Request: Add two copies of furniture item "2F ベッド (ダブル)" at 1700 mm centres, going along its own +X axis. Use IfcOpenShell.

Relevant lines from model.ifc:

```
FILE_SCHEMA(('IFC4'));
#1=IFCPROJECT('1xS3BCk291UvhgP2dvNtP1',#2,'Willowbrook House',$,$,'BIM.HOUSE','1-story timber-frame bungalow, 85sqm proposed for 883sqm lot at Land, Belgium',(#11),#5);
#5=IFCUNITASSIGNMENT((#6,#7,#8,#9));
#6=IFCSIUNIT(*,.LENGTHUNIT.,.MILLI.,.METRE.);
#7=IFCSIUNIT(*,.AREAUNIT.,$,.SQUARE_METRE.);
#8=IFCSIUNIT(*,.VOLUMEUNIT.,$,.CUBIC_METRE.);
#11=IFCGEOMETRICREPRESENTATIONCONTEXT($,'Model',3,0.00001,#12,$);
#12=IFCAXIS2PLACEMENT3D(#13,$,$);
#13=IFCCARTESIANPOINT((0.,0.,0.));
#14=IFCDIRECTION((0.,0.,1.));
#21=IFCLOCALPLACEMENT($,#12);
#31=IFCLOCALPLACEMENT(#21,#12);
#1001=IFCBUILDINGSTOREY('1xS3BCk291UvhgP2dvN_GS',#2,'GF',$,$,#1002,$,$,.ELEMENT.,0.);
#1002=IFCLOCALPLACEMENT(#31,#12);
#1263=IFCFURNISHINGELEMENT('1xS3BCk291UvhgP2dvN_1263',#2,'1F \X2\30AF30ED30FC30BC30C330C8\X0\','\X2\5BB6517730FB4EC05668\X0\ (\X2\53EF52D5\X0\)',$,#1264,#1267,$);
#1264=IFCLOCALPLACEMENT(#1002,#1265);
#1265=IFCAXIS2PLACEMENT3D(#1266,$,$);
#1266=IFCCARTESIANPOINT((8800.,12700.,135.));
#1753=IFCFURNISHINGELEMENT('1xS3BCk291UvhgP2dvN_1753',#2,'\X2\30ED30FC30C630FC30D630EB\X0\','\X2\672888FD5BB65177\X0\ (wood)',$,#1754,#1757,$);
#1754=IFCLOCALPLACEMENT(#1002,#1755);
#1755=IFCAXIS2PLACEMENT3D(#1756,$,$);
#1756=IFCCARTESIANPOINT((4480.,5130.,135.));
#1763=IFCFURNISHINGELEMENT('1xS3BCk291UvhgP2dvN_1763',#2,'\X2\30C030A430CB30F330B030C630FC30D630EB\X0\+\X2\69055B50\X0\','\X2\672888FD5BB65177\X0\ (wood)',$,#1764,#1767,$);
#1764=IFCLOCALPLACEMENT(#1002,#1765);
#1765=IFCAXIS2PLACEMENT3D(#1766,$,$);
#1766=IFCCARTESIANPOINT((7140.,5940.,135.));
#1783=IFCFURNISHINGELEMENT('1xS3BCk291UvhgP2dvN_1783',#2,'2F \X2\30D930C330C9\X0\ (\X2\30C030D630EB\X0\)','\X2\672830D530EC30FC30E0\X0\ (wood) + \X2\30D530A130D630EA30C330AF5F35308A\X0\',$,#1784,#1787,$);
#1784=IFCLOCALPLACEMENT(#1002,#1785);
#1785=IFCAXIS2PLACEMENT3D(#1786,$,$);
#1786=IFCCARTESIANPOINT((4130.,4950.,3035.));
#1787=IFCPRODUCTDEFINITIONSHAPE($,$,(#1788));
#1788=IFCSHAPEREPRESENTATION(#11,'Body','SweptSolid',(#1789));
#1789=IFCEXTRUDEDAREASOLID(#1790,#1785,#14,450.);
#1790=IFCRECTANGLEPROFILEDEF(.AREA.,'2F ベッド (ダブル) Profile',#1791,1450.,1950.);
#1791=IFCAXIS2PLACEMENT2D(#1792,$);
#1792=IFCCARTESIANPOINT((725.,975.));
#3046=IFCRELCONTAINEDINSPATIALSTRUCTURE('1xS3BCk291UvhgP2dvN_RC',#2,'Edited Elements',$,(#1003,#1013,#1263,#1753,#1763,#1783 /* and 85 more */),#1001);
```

```python
import ifcopenshell
import ifcopenshell.api.geometry
import ifcopenshell.api.root
import ifcopenshell.util.element
import ifcopenshell.util.placement

model = ifcopenshell.open("model.ifc")


def reuse_history(source, copy):
    """copy_class also copies each property set's owner history, people and application; keep the originals."""
    for rel in copy.IsDefinedBy:
        if rel.is_a("IfcRelDefinesByProperties") and (history := rel.RelatingPropertyDefinition.OwnerHistory):
            rel.RelatingPropertyDefinition.OwnerHistory = source.OwnerHistory
            ifcopenshell.util.element.remove_deep2(model, history)


source = model.by_id(1783)
base = ifcopenshell.util.placement.get_local_placement(source.ObjectPlacement)
step = base[:3, 0] * 1700.0

for i in range(1, 3):
    copy = ifcopenshell.api.root.copy_class(model, product=source)
    copy.Representation = ifcopenshell.util.element.copy_deep(
        model, source.Representation, exclude=["IfcGeometricRepresentationContext", "IfcRepresentationMap"]
    )
    reuse_history(source, copy)
    matrix = base.copy()
    matrix[:3, 3] += i * step
    print("added at", matrix[:3, 3].round(3) + 0.0)
    ifcopenshell.api.geometry.edit_object_placement(model, product=copy, matrix=matrix, is_si=False)

model.write("model_updated.ifc")
```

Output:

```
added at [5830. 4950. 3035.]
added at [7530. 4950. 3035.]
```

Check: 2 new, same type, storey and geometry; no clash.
